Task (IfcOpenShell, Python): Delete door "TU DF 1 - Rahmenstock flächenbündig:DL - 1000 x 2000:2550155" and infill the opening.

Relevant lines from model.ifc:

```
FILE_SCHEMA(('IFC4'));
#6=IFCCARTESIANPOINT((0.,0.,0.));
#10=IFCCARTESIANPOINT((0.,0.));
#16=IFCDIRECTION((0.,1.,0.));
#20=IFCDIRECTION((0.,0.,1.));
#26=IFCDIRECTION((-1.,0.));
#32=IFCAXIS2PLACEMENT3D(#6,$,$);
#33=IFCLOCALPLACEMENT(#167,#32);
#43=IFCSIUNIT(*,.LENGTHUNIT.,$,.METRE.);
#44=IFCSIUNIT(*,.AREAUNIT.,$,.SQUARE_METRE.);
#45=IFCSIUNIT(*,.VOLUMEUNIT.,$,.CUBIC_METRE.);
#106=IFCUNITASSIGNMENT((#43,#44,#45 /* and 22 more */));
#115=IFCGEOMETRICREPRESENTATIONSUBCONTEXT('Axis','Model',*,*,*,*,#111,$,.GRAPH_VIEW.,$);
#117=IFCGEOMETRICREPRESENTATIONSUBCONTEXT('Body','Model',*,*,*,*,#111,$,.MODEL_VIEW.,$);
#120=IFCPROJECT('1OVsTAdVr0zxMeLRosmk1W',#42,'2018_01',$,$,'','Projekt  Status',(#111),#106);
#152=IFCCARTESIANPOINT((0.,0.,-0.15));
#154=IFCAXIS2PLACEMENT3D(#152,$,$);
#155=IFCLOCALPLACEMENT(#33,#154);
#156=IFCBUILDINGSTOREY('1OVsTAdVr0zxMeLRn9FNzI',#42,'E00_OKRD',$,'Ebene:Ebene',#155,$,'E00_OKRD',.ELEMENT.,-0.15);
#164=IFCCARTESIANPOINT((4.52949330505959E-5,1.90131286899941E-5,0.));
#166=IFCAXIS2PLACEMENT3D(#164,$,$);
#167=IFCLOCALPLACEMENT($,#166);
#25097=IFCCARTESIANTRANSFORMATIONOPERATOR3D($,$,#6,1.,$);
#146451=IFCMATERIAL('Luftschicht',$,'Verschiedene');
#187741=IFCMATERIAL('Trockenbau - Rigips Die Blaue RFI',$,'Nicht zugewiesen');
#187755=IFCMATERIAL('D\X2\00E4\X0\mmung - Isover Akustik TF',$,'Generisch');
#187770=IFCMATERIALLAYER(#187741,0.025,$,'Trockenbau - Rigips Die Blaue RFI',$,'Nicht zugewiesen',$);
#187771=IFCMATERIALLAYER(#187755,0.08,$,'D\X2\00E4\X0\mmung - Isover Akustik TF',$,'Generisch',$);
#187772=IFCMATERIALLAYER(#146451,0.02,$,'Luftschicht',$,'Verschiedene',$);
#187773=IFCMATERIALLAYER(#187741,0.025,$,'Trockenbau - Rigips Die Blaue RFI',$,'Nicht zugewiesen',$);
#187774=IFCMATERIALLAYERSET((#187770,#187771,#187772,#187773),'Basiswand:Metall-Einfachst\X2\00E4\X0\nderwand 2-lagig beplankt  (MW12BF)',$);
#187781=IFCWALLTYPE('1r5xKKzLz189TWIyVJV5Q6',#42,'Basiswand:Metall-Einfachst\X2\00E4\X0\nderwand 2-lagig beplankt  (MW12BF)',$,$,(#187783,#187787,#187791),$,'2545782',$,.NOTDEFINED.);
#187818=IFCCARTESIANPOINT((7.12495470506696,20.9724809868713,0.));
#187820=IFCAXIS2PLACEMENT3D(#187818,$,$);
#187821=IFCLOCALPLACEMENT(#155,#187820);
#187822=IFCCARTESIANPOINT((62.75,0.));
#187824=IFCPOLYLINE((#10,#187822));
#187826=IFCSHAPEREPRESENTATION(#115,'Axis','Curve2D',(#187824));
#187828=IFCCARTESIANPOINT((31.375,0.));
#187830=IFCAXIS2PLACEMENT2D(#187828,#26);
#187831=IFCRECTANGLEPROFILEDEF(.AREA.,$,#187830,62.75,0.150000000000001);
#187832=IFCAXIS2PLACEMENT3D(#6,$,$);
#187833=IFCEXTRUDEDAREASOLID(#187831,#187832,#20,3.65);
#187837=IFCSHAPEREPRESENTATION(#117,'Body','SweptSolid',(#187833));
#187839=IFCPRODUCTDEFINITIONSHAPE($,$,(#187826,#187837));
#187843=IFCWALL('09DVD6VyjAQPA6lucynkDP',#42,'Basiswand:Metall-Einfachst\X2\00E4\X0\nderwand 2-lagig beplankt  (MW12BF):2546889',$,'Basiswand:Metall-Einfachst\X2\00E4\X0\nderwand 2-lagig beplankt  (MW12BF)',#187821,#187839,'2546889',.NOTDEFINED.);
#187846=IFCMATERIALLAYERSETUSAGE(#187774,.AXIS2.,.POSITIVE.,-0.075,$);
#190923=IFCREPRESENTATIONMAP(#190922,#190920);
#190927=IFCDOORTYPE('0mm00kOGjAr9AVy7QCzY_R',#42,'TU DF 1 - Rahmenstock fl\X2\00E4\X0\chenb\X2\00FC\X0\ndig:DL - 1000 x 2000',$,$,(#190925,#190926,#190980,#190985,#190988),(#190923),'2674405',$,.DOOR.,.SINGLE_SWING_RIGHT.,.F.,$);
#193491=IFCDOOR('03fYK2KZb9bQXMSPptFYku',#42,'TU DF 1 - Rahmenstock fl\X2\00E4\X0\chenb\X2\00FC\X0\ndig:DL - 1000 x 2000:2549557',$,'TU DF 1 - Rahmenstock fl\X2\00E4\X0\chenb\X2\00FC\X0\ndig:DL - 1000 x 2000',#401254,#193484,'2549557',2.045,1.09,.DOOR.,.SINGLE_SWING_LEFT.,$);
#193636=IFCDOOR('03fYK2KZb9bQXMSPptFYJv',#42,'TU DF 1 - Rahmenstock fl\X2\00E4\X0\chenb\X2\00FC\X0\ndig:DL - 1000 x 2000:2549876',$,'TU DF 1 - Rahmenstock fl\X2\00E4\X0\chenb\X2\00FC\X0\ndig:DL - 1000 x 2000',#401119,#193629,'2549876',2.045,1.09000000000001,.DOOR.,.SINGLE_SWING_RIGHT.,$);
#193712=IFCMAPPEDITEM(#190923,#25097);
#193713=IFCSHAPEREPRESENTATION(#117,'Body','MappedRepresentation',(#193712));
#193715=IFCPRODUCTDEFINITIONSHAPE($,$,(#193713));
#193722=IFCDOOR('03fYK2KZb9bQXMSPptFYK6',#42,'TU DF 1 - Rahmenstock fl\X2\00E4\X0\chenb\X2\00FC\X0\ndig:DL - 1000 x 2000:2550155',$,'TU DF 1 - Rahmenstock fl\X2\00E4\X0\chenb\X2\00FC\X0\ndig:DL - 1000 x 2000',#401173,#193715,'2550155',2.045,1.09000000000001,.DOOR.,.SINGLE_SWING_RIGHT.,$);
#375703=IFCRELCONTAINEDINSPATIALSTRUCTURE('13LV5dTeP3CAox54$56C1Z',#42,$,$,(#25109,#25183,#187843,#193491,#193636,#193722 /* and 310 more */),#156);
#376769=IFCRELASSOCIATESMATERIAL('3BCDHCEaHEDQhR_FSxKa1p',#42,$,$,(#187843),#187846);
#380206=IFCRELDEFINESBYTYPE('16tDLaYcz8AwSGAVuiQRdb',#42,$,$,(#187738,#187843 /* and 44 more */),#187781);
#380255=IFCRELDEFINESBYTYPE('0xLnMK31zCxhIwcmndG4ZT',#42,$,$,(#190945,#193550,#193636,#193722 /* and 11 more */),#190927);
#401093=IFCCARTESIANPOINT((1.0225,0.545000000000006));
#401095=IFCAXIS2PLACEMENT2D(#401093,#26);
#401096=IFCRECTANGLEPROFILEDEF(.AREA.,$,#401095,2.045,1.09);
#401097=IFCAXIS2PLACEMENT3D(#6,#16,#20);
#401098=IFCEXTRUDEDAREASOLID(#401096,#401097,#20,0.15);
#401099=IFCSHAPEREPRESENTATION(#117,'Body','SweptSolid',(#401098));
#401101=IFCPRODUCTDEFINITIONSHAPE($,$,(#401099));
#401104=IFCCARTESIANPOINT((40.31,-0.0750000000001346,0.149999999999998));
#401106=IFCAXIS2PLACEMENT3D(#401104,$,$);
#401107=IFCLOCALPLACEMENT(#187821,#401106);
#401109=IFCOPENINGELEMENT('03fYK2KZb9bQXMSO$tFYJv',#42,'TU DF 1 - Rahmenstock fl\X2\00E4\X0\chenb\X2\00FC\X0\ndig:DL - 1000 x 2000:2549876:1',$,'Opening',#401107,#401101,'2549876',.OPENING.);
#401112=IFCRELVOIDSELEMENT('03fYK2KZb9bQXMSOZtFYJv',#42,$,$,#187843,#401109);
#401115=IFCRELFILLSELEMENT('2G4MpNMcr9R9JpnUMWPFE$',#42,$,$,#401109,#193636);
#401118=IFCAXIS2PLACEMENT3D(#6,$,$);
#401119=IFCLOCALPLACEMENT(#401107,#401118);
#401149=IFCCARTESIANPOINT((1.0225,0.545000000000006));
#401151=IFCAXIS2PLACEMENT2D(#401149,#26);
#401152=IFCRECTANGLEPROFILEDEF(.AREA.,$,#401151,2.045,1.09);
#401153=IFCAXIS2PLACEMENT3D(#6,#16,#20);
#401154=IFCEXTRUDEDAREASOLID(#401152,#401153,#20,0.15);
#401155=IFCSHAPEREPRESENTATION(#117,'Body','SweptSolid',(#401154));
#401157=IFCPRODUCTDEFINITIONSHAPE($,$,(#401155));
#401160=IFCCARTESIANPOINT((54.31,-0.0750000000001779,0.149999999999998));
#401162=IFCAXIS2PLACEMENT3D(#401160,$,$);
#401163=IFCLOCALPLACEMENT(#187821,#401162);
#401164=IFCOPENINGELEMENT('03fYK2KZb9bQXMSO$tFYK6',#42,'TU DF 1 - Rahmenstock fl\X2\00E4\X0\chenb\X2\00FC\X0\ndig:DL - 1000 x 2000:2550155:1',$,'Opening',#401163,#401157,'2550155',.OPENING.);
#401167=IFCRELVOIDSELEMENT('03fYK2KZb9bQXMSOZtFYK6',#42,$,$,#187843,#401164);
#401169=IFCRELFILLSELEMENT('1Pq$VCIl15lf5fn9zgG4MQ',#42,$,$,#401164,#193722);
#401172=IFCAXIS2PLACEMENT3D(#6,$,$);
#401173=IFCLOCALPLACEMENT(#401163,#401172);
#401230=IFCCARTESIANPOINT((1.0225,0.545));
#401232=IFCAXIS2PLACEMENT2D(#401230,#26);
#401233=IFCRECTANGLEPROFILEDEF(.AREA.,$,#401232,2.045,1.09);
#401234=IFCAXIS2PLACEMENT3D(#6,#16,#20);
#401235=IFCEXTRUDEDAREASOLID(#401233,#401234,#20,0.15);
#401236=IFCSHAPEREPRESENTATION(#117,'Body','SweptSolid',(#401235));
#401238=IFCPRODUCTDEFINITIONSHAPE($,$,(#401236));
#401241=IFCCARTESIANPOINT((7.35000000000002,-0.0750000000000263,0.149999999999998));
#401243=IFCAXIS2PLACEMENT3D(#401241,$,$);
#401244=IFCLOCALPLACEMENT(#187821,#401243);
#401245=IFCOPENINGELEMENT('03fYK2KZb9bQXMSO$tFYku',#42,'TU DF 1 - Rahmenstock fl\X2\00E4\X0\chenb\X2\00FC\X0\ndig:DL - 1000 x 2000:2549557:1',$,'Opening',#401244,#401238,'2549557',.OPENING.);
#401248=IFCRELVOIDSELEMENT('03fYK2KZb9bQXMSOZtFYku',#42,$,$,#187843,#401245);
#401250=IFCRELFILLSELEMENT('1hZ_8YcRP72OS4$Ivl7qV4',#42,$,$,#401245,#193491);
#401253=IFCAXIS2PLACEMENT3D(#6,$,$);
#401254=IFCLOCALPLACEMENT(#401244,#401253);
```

```python
import ifcopenshell
import ifcopenshell.api.feature
import ifcopenshell.api.root
import ifcopenshell.geom
import ifcopenshell.util.shape

model = ifcopenshell.open("model.ifc")
settings = ifcopenshell.geom.settings()


def volume(element):
    """Net volume in cubic metres, openings subtracted."""
    shape = ifcopenshell.geom.create_shape(settings, element)
    return ifcopenshell.util.shape.get_volume(shape.geometry)


door = model.by_guid("03fYK2KZb9bQXMSPptFYK6")
opening = door.FillsVoids[0].RelatingOpeningElement
wall = opening.VoidsElements[0].RelatingBuildingElement
before = volume(wall)

ifcopenshell.api.root.remove_product(model, product=door)
ifcopenshell.api.feature.remove_feature(model, feature=opening)

after = volume(wall)

print(f"wall volume {before:.3f} -> {after:.3f} m3")

model.write("model_v2.ifc")
```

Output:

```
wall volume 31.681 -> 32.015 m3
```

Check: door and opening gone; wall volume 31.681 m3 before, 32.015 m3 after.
